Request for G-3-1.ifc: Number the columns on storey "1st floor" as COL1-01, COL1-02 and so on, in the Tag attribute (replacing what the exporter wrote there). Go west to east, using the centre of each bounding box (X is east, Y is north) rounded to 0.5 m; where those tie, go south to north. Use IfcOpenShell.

First a look at what the model holds.

```python
import ifcopenshell
import ifcopenshell.util.element
import ifcopenshell.util.placement

model = ifcopenshell.open("G-3-1.ifc")
print(model.schema)
storey = next(s for s in model.by_type("IfcBuildingStorey") if s.Name == "1st floor")
columns = [e for e in ifcopenshell.util.element.get_decomposition(storey) if e.is_a("IfcColumn")]
for e in sorted(columns, key=lambda e: e.id()):
    origin = ifcopenshell.util.placement.get_local_placement(e.ObjectPlacement)[:3, 3]
    print(e.id(), e.Tag, e.Name, origin.round(2) + 0.0, sep=" | ")
```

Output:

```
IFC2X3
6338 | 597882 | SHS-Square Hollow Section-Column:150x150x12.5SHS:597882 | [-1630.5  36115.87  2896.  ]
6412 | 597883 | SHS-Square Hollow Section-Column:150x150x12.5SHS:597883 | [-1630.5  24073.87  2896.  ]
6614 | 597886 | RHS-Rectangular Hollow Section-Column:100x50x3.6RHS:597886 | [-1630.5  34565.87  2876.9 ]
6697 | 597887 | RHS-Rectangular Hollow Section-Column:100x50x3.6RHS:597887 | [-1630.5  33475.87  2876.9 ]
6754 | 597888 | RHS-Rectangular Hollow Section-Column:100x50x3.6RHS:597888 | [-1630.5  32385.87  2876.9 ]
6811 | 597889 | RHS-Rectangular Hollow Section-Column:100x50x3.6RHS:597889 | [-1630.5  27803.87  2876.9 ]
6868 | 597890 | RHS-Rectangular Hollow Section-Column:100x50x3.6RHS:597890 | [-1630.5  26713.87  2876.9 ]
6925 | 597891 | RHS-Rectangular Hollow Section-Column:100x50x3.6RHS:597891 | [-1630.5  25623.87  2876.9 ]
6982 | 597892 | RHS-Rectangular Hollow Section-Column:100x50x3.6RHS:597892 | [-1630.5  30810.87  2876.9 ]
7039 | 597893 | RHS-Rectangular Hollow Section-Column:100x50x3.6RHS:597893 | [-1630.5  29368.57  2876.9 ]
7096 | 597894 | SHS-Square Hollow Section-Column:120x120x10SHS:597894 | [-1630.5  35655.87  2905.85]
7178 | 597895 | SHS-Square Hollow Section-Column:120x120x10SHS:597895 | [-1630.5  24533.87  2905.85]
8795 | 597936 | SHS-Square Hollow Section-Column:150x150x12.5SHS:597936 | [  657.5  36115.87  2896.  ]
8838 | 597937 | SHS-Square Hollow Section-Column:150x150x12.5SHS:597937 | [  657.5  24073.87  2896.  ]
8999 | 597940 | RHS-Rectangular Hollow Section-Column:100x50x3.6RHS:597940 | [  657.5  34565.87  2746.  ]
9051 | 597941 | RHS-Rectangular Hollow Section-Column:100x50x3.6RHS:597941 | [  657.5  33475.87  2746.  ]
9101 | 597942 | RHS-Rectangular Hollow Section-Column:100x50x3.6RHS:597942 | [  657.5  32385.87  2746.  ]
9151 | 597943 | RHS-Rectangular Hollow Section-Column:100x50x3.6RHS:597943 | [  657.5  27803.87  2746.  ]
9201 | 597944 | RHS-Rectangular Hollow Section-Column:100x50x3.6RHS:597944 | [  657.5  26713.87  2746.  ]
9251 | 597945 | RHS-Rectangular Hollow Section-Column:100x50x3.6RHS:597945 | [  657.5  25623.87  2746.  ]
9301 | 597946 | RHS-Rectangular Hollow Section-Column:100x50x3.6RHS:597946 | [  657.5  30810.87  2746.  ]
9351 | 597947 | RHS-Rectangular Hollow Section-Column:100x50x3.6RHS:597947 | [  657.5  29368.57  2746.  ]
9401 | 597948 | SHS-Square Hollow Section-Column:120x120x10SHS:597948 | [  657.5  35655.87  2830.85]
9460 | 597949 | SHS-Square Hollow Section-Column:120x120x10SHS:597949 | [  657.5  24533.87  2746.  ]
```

```python
import ifcopenshell
import ifcopenshell.geom
import ifcopenshell.util.element
import ifcopenshell.util.shape

model = ifcopenshell.open("G-3-1.ifc")
settings = ifcopenshell.geom.settings()
settings.set("use-world-coords", True)


def centre(element):
    shape = ifcopenshell.geom.create_shape(settings, element)
    return ifcopenshell.util.shape.get_bbox_centroid(shape.geometry)


storey = next(s for s in model.by_type("IfcBuildingStorey") if s.Name == "1st floor")
columns = [e for e in ifcopenshell.util.element.get_decomposition(storey) if e.is_a("IfcColumn")]

# Insertion points can sit at a corner or the storey origin, so sort by the geometry (in metres).
centres = {e: centre(e) for e in columns}
columns.sort(key=lambda e: (round(centres[e][0] / 0.5), centres[e][1]))

for i, e in enumerate(columns, start=1):
    number = f"COL1-{i:02d}"
    e.Tag = number
    print(e.id(), number)

model.write("G-3-1-out.ifc")
```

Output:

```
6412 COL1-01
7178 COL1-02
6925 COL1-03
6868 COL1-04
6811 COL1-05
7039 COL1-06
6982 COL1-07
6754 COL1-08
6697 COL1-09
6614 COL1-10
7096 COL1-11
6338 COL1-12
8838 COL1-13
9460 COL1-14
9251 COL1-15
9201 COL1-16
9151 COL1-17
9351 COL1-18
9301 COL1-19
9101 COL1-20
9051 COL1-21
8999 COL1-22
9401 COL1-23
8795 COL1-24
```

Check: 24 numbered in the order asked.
